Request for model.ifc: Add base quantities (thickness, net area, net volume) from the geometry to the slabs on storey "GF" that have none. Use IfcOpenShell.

First a look at what the model holds.

```python
import ifcopenshell
import ifcopenshell.util.element
import ifcopenshell.util.unit

model = ifcopenshell.open("model.ifc")
print(model.schema)
for unit_type in ("LENGTHUNIT", "AREAUNIT", "VOLUMEUNIT"):
    print(unit_type, ifcopenshell.util.unit.calculate_unit_scale(model, unit_type))
storey = next(s for s in model.by_type("IfcBuildingStorey") if s.Name == "GF")
slabs = [e for e in ifcopenshell.util.element.get_decomposition(storey) if e.is_a("IfcSlab")]
for e in sorted(slabs, key=lambda e: e.id()):
    print(e.id(), e.is_a(), e.Name, list(ifcopenshell.util.element.get_psets(e, qtos_only=True)), sep=" | ")
```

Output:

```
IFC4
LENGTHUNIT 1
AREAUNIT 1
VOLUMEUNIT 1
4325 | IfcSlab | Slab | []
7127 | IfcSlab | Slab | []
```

```python
import ifcopenshell
import ifcopenshell.api.pset
import ifcopenshell.geom
import ifcopenshell.util.element
import ifcopenshell.util.shape
import ifcopenshell.util.unit

model = ifcopenshell.open("model.ifc")
unit_scale = ifcopenshell.util.unit.calculate_unit_scale(model)
area_scale = ifcopenshell.util.unit.calculate_unit_scale(model, "AREAUNIT")
volume_scale = ifcopenshell.util.unit.calculate_unit_scale(model, "VOLUMEUNIT")
settings = ifcopenshell.geom.settings()

storey = next(s for s in model.by_type("IfcBuildingStorey") if s.Name == "GF")
slabs = [e for e in ifcopenshell.util.element.get_decomposition(storey) if e.is_a("IfcSlab")]

for e in sorted(slabs, key=lambda e: e.id()):
    if ifcopenshell.util.element.get_psets(e, qtos_only=True, should_inherit=False):
        continue
    # Geometry comes back in metres, in the element's own axes.
    shape = ifcopenshell.geom.create_shape(settings, e)
    values = {
        "Width": ifcopenshell.util.shape.get_z(shape.geometry) / unit_scale,
        "NetArea": ifcopenshell.util.shape.get_footprint_area(shape.geometry) / area_scale,
        "NetVolume": ifcopenshell.util.shape.get_volume(shape.geometry) / volume_scale,
    }
    qto = ifcopenshell.api.pset.add_qto(model, product=e, name="Qto_SlabBaseQuantities")
    ifcopenshell.api.pset.edit_qto(model, qto=qto, properties=values)
    print(e.id(), {k: round(v, 3) for k, v in values.items()})

model.write("model-out.ifc")
```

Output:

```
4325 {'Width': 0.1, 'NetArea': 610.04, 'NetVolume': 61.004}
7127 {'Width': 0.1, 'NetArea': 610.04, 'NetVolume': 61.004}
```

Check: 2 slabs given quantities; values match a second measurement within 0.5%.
